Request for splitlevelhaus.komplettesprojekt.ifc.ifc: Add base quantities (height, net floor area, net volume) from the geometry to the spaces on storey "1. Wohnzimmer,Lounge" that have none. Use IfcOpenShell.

First a look at what the model holds.

```python
import ifcopenshell
import ifcopenshell.util.element
import ifcopenshell.util.unit

model = ifcopenshell.open("splitlevelhaus.komplettesprojekt.ifc.ifc")
print(model.schema)
for unit_type in ("LENGTHUNIT", "AREAUNIT", "VOLUMEUNIT"):
    print(unit_type, ifcopenshell.util.unit.calculate_unit_scale(model, unit_type))
storey = next(s for s in model.by_type("IfcBuildingStorey") if s.Name == "1. Wohnzimmer,Lounge")
spaces = [e for e in ifcopenshell.util.element.get_decomposition(storey) if e.is_a("IfcSpace")]
for e in sorted(spaces, key=lambda e: e.id()):
    print(e.id(), e.is_a(), e.Name, list(ifcopenshell.util.element.get_psets(e, qtos_only=True)), sep=" | ")
```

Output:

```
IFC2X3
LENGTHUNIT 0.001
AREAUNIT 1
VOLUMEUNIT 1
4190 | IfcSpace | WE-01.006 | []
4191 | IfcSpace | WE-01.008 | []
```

```python
import ifcopenshell
import ifcopenshell.api.pset
import ifcopenshell.geom
import ifcopenshell.util.element
import ifcopenshell.util.shape
import ifcopenshell.util.unit

model = ifcopenshell.open("splitlevelhaus.komplettesprojekt.ifc.ifc")
unit_scale = ifcopenshell.util.unit.calculate_unit_scale(model)
area_scale = ifcopenshell.util.unit.calculate_unit_scale(model, "AREAUNIT")
volume_scale = ifcopenshell.util.unit.calculate_unit_scale(model, "VOLUMEUNIT")
settings = ifcopenshell.geom.settings()

storey = next(s for s in model.by_type("IfcBuildingStorey") if s.Name == "1. Wohnzimmer,Lounge")
spaces = [e for e in ifcopenshell.util.element.get_decomposition(storey) if e.is_a("IfcSpace")]

for e in sorted(spaces, key=lambda e: e.id()):
    if ifcopenshell.util.element.get_psets(e, qtos_only=True, should_inherit=False):
        continue
    # Geometry comes back in metres, in the element's own axes.
    shape = ifcopenshell.geom.create_shape(settings, e)
    values = {
        "Height": ifcopenshell.util.shape.get_z(shape.geometry) / unit_scale,
        "NetFloorArea": ifcopenshell.util.shape.get_footprint_area(shape.geometry) / area_scale,
        "NetVolume": ifcopenshell.util.shape.get_volume(shape.geometry) / volume_scale,
    }
    qto = ifcopenshell.api.pset.add_qto(model, product=e, name="BaseQuantities")
    ifcopenshell.api.pset.edit_qto(model, qto=qto, properties=values)
    print(e.id(), {k: round(v, 3) for k, v in values.items()})

model.write("splitlevelhaus.komplettesprojekt.ifc_rev.ifc")
```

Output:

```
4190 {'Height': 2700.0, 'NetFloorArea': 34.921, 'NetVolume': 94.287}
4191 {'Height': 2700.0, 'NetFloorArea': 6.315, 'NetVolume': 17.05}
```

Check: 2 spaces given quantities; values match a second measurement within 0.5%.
